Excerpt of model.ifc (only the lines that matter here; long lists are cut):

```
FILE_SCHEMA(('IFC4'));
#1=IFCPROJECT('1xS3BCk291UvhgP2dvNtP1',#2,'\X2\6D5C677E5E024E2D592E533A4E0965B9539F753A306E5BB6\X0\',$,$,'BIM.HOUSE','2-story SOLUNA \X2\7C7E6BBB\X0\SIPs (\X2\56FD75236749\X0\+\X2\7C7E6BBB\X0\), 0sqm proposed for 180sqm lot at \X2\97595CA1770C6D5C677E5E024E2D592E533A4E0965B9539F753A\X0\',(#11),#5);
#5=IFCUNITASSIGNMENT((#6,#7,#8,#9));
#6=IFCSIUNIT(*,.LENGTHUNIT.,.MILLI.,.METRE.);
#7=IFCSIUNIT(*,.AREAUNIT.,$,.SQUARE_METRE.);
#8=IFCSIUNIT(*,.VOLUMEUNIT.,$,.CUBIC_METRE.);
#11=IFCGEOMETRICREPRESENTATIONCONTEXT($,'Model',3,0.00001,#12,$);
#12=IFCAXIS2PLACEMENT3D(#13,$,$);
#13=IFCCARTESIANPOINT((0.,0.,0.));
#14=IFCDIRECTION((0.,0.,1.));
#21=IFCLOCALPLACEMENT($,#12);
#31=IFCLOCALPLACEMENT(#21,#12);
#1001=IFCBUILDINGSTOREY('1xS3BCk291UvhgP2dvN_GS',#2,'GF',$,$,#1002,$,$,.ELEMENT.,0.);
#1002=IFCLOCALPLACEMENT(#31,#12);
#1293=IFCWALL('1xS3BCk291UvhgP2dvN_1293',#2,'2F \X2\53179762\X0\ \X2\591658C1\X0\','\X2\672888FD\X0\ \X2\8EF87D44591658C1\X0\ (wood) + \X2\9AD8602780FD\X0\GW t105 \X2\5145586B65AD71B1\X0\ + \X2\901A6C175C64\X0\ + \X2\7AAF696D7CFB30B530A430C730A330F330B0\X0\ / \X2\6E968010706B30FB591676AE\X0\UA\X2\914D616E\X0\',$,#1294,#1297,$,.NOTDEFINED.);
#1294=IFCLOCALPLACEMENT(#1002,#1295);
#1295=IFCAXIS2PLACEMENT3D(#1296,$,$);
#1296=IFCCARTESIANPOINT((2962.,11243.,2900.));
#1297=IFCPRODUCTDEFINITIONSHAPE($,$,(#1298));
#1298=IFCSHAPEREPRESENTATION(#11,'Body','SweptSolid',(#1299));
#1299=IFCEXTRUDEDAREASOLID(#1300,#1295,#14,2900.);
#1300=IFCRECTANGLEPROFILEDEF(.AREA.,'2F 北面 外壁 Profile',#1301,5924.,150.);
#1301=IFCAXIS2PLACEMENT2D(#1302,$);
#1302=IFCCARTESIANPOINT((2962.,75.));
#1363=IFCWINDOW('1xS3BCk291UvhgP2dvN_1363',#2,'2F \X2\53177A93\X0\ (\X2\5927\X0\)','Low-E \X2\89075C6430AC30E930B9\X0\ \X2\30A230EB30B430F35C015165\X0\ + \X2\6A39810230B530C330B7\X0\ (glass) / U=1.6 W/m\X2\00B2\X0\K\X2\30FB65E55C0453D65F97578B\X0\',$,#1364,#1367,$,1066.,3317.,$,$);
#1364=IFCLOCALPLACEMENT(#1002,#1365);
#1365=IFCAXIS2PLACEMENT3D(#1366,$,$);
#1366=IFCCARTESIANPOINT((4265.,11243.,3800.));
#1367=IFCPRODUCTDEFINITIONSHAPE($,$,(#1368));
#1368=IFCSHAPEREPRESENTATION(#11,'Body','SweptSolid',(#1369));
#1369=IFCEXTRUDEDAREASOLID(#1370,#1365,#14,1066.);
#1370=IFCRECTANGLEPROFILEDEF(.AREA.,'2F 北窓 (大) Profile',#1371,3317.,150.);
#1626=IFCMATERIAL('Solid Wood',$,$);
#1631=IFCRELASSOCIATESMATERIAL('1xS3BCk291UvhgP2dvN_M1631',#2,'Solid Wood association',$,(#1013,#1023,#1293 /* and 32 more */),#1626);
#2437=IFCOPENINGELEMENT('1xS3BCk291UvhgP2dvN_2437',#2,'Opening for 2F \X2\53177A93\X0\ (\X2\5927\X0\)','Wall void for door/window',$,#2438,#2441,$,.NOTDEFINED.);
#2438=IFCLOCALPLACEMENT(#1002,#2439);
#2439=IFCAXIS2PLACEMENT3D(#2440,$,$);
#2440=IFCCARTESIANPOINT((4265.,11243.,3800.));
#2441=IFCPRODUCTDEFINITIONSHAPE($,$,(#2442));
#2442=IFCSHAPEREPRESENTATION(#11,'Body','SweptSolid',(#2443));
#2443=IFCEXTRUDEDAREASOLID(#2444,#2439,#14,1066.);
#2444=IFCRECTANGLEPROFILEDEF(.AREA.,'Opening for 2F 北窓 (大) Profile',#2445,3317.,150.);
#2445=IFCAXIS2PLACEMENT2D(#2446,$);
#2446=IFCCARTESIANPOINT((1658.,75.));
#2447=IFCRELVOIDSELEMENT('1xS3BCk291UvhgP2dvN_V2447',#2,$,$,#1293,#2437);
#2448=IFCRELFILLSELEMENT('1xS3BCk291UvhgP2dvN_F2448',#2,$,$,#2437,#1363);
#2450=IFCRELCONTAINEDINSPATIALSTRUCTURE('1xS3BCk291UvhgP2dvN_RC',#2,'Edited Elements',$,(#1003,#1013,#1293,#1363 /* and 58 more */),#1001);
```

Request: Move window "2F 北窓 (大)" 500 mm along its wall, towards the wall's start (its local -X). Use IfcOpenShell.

```python
import ifcopenshell
import ifcopenshell.api.geometry
import ifcopenshell.util.placement

model = ifcopenshell.open("model.ifc")

window = model.by_guid("1xS3BCk291UvhgP2dvN_1363")
opening = window.FillsVoids[0].RelatingOpeningElement
wall = opening.VoidsElements[0].RelatingBuildingElement

wall_matrix = ifcopenshell.util.placement.get_local_placement(wall.ObjectPlacement)
shift = wall_matrix[:3, 0] * -500.0
before = ifcopenshell.util.placement.get_local_placement(window.ObjectPlacement)[:3, 3].copy()

# The window is not placed relative to its opening, so move both.
for product in (opening, window):
    matrix = ifcopenshell.util.placement.get_local_placement(product.ObjectPlacement)
    matrix[:3, 3] += shift
    ifcopenshell.api.geometry.edit_object_placement(model, product=product, matrix=matrix, is_si=False)

after = ifcopenshell.util.placement.get_local_placement(window.ObjectPlacement)[:3, 3]
print("window moved by", (after - before).round(3) + 0.0)

model.write("model_rev.ifc")
```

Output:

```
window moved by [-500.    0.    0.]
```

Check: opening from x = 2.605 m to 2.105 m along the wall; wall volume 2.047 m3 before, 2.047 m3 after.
